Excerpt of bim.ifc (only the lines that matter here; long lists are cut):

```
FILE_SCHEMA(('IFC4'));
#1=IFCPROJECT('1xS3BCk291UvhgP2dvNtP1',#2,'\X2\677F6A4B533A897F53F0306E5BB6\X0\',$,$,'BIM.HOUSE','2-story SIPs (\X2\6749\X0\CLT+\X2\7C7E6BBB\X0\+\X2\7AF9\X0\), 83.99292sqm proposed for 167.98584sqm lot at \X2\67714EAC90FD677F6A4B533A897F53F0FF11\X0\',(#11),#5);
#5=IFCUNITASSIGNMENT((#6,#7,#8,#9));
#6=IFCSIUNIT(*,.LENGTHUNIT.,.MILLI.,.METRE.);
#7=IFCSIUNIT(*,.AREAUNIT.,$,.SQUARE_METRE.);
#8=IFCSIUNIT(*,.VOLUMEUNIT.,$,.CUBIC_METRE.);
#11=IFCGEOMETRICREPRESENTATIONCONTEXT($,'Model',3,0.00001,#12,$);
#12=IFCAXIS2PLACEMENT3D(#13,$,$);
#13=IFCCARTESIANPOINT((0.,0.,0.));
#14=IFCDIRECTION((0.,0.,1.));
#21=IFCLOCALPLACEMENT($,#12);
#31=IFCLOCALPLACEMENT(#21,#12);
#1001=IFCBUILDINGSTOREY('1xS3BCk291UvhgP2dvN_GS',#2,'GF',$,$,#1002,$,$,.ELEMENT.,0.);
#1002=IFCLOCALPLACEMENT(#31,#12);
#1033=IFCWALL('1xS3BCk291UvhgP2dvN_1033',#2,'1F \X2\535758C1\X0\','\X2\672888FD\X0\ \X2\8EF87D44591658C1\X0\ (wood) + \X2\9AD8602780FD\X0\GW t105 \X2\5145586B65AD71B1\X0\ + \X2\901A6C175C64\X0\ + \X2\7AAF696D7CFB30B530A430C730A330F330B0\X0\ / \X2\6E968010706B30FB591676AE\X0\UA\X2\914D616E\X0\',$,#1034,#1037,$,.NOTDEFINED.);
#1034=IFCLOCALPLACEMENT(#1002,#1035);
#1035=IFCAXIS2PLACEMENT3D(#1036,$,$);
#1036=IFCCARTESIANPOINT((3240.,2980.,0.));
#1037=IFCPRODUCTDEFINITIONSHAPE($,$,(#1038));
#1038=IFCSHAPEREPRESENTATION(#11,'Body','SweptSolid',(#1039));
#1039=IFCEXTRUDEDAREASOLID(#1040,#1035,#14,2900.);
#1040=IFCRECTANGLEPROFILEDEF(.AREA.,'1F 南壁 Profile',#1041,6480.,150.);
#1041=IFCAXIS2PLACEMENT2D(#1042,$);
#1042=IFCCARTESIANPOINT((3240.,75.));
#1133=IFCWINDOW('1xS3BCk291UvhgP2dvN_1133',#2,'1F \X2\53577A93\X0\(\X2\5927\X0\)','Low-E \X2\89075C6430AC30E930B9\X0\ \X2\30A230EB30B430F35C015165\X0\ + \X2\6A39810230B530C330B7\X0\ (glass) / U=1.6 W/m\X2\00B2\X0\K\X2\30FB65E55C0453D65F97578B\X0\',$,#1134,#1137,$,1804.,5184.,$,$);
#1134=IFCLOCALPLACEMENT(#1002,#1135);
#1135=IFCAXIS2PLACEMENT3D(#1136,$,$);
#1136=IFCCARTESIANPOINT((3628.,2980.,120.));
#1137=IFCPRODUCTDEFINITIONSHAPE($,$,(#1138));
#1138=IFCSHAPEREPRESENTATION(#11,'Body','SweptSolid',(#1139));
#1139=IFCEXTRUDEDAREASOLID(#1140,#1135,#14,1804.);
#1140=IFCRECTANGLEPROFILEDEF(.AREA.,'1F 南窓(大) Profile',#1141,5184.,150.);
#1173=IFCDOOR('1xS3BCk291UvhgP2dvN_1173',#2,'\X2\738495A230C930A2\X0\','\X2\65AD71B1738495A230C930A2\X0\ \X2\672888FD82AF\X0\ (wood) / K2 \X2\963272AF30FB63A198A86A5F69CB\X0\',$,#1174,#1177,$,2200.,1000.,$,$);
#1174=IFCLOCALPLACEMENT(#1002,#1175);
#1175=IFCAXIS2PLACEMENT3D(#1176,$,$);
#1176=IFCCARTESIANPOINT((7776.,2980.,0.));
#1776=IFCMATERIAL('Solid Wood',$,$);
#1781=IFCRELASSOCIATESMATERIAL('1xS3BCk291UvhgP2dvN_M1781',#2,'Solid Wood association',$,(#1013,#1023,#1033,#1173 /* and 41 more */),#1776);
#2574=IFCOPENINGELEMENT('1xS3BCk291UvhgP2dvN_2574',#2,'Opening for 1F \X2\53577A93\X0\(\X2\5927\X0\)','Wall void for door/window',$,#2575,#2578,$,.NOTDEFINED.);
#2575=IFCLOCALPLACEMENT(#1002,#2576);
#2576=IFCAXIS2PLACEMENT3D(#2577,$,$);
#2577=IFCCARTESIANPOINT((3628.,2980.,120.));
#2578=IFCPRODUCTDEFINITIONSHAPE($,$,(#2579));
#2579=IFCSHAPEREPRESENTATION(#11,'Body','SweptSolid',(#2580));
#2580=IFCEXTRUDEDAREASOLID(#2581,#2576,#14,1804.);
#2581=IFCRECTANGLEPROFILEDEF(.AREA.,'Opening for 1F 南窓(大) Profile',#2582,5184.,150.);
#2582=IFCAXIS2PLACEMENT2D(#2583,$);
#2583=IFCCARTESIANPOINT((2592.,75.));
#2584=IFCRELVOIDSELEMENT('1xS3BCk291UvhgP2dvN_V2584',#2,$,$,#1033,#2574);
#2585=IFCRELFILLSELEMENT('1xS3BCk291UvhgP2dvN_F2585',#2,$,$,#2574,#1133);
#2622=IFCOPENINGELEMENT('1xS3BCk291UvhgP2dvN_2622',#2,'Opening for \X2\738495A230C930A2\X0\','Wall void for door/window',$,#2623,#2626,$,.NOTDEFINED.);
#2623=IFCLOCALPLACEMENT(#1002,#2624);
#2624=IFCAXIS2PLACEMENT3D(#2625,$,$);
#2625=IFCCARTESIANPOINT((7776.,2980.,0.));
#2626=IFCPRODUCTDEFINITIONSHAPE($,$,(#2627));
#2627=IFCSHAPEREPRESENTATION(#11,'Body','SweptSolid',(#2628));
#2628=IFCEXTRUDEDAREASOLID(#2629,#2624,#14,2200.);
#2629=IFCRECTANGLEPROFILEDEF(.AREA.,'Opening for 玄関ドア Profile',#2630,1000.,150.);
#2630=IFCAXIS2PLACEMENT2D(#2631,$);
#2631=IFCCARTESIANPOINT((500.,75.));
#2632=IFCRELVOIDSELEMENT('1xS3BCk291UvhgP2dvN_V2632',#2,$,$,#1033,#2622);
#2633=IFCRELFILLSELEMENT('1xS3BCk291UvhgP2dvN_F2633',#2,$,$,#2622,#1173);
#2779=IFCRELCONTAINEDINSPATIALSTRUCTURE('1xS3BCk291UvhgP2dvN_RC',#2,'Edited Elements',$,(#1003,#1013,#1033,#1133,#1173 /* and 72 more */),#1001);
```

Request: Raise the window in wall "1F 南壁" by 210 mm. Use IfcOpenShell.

```python
import numpy as np
import ifcopenshell
import ifcopenshell.api.geometry
import ifcopenshell.util.placement
import ifcopenshell.util.unit

model = ifcopenshell.open("bim.ifc")
unit_scale = ifcopenshell.util.unit.calculate_unit_scale(model)

window = model.by_id(1133)
opening = window.FillsVoids[0].RelatingOpeningElement
dz = 0.21 / unit_scale

shift = np.array([0.0, 0.0, dz])
# The window is not placed relative to its opening, so move both.
for product in (opening, window):
    matrix = ifcopenshell.util.placement.get_local_placement(product.ObjectPlacement)
    matrix[:3, 3] += shift
    ifcopenshell.api.geometry.edit_object_placement(model, product=product, matrix=matrix, is_si=False)

print(f"moved by {dz * unit_scale:+.3f} m")

model.write("bim_edited.ifc")
```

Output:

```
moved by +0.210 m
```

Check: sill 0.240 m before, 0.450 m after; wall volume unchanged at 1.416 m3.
